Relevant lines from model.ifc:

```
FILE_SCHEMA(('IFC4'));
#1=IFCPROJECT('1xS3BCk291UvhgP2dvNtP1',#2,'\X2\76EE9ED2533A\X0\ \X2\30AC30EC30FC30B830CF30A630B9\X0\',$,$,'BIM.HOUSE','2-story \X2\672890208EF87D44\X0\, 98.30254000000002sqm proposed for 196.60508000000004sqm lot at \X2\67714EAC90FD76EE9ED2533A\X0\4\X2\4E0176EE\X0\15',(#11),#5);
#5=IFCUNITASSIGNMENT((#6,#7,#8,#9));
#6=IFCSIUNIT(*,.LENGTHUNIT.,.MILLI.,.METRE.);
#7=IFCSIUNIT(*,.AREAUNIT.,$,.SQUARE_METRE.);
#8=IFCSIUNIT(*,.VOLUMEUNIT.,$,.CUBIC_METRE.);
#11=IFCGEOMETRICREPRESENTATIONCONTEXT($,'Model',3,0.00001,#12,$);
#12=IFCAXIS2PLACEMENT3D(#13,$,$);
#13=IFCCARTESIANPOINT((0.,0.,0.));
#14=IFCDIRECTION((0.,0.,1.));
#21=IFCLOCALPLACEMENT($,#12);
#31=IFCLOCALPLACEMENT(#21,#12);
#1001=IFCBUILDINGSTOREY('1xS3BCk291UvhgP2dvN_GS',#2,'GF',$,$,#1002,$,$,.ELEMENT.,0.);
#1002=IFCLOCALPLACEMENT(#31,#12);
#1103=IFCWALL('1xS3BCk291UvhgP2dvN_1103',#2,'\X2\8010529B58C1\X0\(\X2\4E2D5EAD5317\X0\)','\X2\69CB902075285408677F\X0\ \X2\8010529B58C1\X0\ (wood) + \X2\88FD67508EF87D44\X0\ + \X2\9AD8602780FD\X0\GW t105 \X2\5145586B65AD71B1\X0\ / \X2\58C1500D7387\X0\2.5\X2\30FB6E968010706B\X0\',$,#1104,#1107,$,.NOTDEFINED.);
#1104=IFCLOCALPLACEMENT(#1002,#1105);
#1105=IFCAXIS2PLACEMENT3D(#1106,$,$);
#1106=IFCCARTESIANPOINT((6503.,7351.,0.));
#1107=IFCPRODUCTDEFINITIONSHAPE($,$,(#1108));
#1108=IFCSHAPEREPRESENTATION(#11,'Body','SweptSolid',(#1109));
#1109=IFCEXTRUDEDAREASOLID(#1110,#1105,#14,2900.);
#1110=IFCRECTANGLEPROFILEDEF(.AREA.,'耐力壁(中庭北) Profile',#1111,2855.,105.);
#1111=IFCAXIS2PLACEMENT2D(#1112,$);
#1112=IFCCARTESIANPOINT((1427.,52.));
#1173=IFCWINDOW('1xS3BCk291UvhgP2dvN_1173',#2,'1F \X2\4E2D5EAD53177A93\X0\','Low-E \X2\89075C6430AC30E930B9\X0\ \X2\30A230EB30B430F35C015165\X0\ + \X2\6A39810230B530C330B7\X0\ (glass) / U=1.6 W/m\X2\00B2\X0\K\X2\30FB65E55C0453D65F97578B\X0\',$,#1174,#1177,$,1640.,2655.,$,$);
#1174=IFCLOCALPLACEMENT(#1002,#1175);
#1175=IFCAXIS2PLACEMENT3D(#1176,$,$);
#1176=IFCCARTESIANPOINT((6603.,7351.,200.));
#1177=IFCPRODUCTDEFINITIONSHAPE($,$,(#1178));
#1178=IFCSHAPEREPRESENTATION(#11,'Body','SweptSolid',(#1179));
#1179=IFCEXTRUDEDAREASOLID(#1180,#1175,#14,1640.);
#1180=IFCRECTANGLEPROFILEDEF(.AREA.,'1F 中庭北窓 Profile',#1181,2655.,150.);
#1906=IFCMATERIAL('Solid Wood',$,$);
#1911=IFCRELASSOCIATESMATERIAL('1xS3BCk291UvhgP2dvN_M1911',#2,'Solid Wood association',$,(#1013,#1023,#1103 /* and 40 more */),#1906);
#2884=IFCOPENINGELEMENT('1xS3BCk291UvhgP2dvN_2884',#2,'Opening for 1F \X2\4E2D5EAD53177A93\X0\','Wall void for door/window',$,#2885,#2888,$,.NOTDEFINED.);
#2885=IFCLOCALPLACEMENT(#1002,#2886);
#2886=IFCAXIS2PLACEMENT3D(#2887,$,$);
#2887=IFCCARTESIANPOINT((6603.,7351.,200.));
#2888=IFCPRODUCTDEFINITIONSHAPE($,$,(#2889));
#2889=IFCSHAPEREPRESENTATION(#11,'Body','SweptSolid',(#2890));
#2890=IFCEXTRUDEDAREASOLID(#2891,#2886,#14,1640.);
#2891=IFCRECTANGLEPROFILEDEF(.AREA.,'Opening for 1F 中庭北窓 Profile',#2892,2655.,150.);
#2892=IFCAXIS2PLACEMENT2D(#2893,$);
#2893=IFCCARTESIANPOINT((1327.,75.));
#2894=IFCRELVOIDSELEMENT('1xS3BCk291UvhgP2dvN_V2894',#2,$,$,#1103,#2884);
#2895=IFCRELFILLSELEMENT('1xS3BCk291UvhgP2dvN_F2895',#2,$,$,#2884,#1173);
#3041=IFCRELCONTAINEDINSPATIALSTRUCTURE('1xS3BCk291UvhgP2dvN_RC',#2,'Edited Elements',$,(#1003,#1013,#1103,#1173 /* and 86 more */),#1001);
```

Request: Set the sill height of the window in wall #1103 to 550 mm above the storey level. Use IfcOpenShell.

```python
import numpy as np
import ifcopenshell
import ifcopenshell.api.geometry
import ifcopenshell.geom
import ifcopenshell.util.element
import ifcopenshell.util.placement
import ifcopenshell.util.shape
import ifcopenshell.util.unit

model = ifcopenshell.open("model.ifc")
unit_scale = ifcopenshell.util.unit.calculate_unit_scale(model)

window = model.by_guid("1xS3BCk291UvhgP2dvN_1173")
opening = window.FillsVoids[0].RelatingOpeningElement
storey = ifcopenshell.util.element.get_container(window, ifc_class="IfcBuildingStorey")
level = ifcopenshell.util.placement.get_local_placement(storey.ObjectPlacement)[2, 3]

# The opening's origin need not be at the sill, so measure its lowest point.
shape = ifcopenshell.geom.create_shape(ifcopenshell.geom.settings(), opening)
bottom = ifcopenshell.util.shape.get_shape_bottom_elevation(shape, shape.geometry) / unit_scale
dz = level + 550.0 - bottom

shift = np.array([0.0, 0.0, dz])
# The window is not placed relative to its opening, so move both.
for product in (opening, window):
    matrix = ifcopenshell.util.placement.get_local_placement(product.ObjectPlacement)
    matrix[:3, 3] += shift
    ifcopenshell.api.geometry.edit_object_placement(model, product=product, matrix=matrix, is_si=False)

print(f"moved by {dz * unit_scale:+.3f} m")

model.write("model-out.ifc")
```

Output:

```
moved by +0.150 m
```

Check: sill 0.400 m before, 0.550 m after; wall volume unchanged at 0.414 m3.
